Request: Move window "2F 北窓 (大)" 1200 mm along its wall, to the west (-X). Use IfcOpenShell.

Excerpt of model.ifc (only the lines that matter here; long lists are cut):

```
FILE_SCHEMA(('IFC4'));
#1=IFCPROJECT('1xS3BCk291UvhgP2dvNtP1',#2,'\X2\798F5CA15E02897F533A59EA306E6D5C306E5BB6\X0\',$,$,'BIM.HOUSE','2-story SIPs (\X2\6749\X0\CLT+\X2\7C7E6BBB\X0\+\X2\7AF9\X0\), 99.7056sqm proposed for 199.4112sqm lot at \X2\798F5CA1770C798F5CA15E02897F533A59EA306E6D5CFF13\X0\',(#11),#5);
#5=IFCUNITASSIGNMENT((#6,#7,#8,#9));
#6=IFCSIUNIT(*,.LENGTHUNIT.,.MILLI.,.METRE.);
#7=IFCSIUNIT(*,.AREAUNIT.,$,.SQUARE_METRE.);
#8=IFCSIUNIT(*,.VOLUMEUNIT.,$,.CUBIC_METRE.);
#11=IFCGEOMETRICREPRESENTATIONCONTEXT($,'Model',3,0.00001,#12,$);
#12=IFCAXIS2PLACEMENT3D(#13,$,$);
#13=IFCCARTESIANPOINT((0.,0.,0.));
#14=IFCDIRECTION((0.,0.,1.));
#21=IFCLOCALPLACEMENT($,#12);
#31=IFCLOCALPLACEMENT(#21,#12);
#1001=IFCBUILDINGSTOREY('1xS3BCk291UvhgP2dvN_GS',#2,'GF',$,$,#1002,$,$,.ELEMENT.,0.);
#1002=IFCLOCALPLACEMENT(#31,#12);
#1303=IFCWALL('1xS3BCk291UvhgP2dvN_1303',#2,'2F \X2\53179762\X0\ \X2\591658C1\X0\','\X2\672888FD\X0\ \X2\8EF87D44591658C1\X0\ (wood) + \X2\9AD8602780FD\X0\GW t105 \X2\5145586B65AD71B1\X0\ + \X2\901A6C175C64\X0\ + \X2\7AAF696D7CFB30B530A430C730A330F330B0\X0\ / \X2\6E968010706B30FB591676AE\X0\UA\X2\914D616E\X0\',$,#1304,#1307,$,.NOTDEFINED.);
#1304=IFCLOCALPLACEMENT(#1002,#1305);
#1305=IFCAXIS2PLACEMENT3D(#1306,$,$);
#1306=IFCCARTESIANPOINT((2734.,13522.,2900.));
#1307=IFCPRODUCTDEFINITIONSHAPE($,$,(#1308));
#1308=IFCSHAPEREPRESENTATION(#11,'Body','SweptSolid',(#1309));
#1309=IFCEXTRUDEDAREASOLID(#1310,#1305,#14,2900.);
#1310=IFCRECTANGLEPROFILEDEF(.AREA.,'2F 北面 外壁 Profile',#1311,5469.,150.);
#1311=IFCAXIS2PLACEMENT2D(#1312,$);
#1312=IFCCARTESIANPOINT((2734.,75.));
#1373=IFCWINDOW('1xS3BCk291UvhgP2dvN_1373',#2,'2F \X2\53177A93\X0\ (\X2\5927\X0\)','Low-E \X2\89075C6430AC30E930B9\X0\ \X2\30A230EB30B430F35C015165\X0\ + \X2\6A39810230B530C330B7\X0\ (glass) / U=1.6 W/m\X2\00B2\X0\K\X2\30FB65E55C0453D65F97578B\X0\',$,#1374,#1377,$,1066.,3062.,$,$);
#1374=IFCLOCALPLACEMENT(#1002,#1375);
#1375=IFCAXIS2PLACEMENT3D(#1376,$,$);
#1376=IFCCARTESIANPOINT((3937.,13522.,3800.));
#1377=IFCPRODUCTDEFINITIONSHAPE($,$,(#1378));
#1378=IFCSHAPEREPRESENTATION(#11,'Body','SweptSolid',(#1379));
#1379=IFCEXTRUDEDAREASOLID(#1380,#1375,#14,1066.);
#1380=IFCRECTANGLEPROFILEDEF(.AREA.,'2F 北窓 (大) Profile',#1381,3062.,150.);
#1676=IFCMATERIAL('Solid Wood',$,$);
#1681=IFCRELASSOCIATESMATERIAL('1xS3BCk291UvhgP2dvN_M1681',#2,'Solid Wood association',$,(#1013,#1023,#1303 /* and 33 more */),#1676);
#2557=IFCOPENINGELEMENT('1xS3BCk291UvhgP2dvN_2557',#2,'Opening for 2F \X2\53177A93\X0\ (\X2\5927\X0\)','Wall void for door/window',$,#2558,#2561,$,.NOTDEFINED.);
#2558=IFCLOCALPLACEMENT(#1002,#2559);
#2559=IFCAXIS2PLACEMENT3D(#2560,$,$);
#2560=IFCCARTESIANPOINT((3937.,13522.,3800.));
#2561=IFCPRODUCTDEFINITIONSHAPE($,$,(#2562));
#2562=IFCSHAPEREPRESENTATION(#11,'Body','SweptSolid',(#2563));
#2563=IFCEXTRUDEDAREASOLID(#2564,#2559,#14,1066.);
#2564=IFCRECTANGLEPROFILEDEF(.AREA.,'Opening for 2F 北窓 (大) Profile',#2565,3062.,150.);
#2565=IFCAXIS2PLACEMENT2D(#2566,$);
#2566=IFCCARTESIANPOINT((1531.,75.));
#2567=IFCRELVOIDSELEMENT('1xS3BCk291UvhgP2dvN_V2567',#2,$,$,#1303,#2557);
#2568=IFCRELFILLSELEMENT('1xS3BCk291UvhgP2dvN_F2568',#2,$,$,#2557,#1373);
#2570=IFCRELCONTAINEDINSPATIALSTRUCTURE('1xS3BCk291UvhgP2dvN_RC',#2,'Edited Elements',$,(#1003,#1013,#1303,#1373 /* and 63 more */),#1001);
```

```python
import ifcopenshell
import ifcopenshell.api.geometry
import ifcopenshell.util.placement
import ifcopenshell.util.unit

model = ifcopenshell.open("model.ifc")
unit_scale = ifcopenshell.util.unit.calculate_unit_scale(model)

window = model.by_guid("1xS3BCk291UvhgP2dvN_1373")
opening = window.FillsVoids[0].RelatingOpeningElement
wall = opening.VoidsElements[0].RelatingBuildingElement

wall_matrix = ifcopenshell.util.placement.get_local_placement(wall.ObjectPlacement)
shift = wall_matrix[:3, 0] * -1.2 / unit_scale
before = ifcopenshell.util.placement.get_local_placement(window.ObjectPlacement)[:3, 3].copy()

# The window is not placed relative to its opening, so move both.
for product in (opening, window):
    matrix = ifcopenshell.util.placement.get_local_placement(product.ObjectPlacement)
    matrix[:3, 3] += shift
    ifcopenshell.api.geometry.edit_object_placement(model, product=product, matrix=matrix, is_si=False)

after = ifcopenshell.util.placement.get_local_placement(window.ObjectPlacement)[:3, 3]
print("window moved by", (after - before).round(3) + 0.0)

model.write("model_edited.ifc")
```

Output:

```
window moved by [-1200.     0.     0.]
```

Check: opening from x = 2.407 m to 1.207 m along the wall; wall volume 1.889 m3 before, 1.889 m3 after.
